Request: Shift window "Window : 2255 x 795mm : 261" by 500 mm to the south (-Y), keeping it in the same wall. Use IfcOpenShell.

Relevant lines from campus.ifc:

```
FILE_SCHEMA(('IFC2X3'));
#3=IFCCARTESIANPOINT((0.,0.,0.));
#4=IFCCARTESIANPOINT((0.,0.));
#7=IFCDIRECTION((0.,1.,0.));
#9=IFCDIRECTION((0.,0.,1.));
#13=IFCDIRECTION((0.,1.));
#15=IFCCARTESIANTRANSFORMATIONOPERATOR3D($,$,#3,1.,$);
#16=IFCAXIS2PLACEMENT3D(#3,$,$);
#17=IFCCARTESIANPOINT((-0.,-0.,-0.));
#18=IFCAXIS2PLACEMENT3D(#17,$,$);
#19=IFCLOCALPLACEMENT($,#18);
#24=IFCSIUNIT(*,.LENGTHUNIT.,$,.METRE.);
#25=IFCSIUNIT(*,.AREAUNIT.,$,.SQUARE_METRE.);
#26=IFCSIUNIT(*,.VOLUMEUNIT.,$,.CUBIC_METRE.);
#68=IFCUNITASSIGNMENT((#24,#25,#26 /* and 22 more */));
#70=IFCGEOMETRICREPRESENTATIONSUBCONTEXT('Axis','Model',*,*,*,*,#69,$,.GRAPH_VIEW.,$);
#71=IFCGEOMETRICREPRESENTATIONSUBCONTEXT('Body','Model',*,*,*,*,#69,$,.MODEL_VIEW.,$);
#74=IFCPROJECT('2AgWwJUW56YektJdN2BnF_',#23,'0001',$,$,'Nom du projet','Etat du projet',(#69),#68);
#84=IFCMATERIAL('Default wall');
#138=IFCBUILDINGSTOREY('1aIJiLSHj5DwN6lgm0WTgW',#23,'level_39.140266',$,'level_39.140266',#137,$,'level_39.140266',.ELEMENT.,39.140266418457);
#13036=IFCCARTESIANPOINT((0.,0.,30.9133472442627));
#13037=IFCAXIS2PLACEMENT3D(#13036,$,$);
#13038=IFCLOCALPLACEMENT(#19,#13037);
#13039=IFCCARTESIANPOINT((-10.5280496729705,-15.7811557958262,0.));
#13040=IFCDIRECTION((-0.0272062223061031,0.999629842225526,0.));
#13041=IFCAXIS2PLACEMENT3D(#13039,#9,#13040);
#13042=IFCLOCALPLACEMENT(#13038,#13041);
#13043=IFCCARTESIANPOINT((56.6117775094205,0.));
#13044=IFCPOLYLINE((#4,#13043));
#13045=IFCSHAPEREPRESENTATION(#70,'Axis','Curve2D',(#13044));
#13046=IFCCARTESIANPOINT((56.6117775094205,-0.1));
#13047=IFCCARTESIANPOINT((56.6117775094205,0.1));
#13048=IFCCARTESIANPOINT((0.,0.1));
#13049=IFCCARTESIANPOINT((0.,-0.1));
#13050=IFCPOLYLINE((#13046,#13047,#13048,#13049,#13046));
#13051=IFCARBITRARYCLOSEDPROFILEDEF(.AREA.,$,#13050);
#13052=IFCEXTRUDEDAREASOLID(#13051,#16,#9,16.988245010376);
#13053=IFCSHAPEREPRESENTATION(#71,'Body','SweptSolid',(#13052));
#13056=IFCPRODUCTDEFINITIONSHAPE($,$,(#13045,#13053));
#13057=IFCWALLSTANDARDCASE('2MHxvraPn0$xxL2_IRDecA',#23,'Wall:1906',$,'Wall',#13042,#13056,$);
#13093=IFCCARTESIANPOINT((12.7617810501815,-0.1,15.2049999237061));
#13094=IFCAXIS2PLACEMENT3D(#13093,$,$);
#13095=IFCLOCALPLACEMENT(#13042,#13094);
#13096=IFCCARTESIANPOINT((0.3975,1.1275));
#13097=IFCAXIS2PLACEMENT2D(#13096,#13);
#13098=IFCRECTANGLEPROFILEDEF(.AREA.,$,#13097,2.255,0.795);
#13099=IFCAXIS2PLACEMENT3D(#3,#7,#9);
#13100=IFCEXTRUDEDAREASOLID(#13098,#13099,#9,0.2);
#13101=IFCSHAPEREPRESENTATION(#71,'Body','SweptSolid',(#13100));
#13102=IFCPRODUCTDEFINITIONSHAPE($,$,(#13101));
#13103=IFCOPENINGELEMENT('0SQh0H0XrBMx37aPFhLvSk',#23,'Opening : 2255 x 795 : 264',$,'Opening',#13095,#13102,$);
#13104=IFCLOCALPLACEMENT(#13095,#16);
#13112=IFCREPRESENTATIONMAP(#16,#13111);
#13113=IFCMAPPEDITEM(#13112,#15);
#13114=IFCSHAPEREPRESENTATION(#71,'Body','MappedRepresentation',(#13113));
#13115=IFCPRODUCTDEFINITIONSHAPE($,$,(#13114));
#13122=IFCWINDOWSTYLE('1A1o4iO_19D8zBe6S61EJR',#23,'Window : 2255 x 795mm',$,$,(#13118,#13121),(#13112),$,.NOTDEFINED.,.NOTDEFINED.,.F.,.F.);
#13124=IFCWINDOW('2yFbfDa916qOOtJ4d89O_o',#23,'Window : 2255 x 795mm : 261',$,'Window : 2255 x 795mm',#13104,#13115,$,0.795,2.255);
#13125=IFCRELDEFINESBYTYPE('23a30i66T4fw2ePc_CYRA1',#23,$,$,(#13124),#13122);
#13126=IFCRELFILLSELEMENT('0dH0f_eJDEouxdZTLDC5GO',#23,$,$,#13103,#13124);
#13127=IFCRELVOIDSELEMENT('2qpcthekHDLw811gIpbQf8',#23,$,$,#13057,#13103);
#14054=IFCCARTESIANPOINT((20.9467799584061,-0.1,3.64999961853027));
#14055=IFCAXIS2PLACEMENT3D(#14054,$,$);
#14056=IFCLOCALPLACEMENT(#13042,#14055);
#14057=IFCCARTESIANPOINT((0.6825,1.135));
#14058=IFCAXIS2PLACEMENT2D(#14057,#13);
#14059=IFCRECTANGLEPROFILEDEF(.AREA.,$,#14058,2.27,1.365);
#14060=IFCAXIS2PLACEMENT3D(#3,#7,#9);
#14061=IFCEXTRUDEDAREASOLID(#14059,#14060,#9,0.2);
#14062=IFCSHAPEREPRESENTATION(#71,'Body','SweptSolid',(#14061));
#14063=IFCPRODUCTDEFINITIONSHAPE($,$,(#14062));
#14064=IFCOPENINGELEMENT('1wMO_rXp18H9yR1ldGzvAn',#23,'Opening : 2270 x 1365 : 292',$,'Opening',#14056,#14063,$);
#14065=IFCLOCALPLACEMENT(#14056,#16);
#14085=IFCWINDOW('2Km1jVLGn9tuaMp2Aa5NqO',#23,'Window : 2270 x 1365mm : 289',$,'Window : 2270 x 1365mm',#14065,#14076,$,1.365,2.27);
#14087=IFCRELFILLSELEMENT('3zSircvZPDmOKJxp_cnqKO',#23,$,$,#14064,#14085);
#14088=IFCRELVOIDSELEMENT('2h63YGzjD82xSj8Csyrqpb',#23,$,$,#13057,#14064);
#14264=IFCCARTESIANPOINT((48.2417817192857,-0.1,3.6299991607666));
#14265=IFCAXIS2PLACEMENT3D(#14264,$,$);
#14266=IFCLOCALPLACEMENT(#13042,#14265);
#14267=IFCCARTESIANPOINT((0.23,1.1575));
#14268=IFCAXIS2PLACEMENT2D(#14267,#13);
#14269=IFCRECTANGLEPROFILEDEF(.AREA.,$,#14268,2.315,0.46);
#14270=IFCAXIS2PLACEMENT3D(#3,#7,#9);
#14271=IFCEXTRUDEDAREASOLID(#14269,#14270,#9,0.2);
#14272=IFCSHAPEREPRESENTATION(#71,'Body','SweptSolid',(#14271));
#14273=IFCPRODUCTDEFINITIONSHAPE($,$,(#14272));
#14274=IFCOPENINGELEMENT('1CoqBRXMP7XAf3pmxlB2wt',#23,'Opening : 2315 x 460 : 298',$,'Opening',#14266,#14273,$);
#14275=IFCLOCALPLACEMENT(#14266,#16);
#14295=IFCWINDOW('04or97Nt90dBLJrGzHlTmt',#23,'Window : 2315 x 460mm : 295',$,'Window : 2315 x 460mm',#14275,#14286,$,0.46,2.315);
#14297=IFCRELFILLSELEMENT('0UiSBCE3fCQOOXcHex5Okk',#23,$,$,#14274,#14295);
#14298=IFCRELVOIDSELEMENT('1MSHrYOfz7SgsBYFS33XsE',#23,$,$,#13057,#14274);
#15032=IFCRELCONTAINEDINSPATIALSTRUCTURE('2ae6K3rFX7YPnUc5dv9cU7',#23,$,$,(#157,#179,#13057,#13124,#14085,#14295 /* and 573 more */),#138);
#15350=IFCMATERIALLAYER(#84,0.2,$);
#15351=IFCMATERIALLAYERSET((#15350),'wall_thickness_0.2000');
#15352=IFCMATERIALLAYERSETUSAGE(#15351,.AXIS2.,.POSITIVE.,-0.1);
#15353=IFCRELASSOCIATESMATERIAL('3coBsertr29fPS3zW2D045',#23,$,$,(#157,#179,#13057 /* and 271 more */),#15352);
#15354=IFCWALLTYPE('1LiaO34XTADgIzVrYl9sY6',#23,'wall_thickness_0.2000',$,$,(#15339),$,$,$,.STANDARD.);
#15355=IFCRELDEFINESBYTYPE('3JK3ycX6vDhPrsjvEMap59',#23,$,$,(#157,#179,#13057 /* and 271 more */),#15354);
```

```python
import ifcopenshell
import ifcopenshell.api.geometry
import ifcopenshell.util.placement

model = ifcopenshell.open("campus.ifc")

window = model.by_guid("2yFbfDa916qOOtJ4d89O_o")
opening = window.FillsVoids[0].RelatingOpeningElement
wall = opening.VoidsElements[0].RelatingBuildingElement

wall_matrix = ifcopenshell.util.placement.get_local_placement(wall.ObjectPlacement)
shift = wall_matrix[:3, 0] * -0.5
before = ifcopenshell.util.placement.get_local_placement(window.ObjectPlacement)[:3, 3].copy()

# The window is placed relative to its opening, so it follows when the opening moves.
matrix = ifcopenshell.util.placement.get_local_placement(opening.ObjectPlacement)
matrix[:3, 3] += shift
ifcopenshell.api.geometry.edit_object_placement(
    model, product=opening, matrix=matrix, is_si=False, should_transform_children=True
)

after = ifcopenshell.util.placement.get_local_placement(window.ObjectPlacement)[:3, 3]
print("window moved by", (after - before).round(3) + 0.0)

model.write("campus_rev.ifc")
```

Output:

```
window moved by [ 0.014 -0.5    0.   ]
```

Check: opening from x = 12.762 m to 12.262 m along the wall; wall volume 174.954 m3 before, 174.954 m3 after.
